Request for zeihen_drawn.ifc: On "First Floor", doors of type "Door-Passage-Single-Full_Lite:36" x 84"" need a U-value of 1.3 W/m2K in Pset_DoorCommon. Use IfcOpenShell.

First a look at what the model holds.

```python
import ifcopenshell
import ifcopenshell.util.element

model = ifcopenshell.open("zeihen_drawn.ifc")
print(model.schema)
storey = next(s for s in model.by_type("IfcBuildingStorey") if s.Name == "First Floor")
doors = [e for e in ifcopenshell.util.element.get_decomposition(storey) if e.is_a("IfcDoor")]
seen = {}
for e in doors:
    element_type = ifcopenshell.util.element.get_type(e)
    key = (element_type.Name if element_type != e and element_type else None, ifcopenshell.util.element.get_pset(e, "Pset_DoorCommon", "ThermalTransmittance"))
    seen[key] = seen.get(key, 0) + 1
for (name, value), count in sorted(seen.items(), key=str):
    print(count, "x", name, "|", value)
```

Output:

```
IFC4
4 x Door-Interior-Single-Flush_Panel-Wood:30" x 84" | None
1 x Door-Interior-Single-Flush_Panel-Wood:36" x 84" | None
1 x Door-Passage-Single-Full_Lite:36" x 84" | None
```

```python
import ifcopenshell
import ifcopenshell.api.pset
import ifcopenshell.util.element

model = ifcopenshell.open("zeihen_drawn.ifc")

storey = next(s for s in model.by_type("IfcBuildingStorey") if s.Name == "First Floor")
doors = [e for e in ifcopenshell.util.element.get_decomposition(storey) if e.is_a("IfcDoor")]

count = 0
for e in doors:
    element_type = ifcopenshell.util.element.get_type(e)
    if element_type in (None, e) or element_type.Name != 'Door-Passage-Single-Full_Lite:36" x 84"':
        continue
    # add_pset returns the element's existing set when there is one.
    pset = ifcopenshell.api.pset.add_pset(model, product=e, name="Pset_DoorCommon")
    ifcopenshell.api.pset.edit_pset(model, pset=pset, properties={"ThermalTransmittance": 1.3})
    count += 1

print(count, "doors updated")

model.write("zeihen_drawn_updated.ifc")
```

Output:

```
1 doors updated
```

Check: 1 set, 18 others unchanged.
